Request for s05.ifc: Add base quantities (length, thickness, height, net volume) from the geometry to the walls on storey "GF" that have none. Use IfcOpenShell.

First a look at what the model holds.

```python
import ifcopenshell
import ifcopenshell.util.element
import ifcopenshell.util.unit

model = ifcopenshell.open("s05.ifc")
print(model.schema)
for unit_type in ("LENGTHUNIT", "AREAUNIT", "VOLUMEUNIT"):
    print(unit_type, ifcopenshell.util.unit.calculate_unit_scale(model, unit_type))
storey = next(s for s in model.by_type("IfcBuildingStorey") if s.Name == "GF")
walls = [e for e in ifcopenshell.util.element.get_decomposition(storey) if e.is_a("IfcWall")]
for e in sorted(walls, key=lambda e: e.id()):
    print(e.id(), e.is_a(), e.Name, list(ifcopenshell.util.element.get_psets(e, qtos_only=True)), sep=" | ")
```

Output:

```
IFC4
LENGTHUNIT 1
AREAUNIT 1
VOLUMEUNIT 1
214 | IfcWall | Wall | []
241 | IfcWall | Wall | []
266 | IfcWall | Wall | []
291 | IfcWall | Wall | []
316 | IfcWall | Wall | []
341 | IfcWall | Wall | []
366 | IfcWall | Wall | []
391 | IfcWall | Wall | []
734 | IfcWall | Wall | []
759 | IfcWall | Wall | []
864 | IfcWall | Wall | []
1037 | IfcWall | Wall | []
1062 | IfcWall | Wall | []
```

```python
import ifcopenshell
import ifcopenshell.api.pset
import ifcopenshell.geom
import ifcopenshell.util.element
import ifcopenshell.util.shape
import ifcopenshell.util.unit

model = ifcopenshell.open("s05.ifc")
unit_scale = ifcopenshell.util.unit.calculate_unit_scale(model)
volume_scale = ifcopenshell.util.unit.calculate_unit_scale(model, "VOLUMEUNIT")
settings = ifcopenshell.geom.settings()

storey = next(s for s in model.by_type("IfcBuildingStorey") if s.Name == "GF")
walls = [e for e in ifcopenshell.util.element.get_decomposition(storey) if e.is_a("IfcWall")]

for e in sorted(walls, key=lambda e: e.id()):
    if ifcopenshell.util.element.get_psets(e, qtos_only=True, should_inherit=False):
        continue
    # Geometry comes back in metres, in the element's own axes.
    shape = ifcopenshell.geom.create_shape(settings, e)
    values = {
        "Length": ifcopenshell.util.shape.get_x(shape.geometry) / unit_scale,
        "Width": ifcopenshell.util.shape.get_y(shape.geometry) / unit_scale,
        "Height": ifcopenshell.util.shape.get_z(shape.geometry) / unit_scale,
        "NetVolume": ifcopenshell.util.shape.get_volume(shape.geometry) / volume_scale,
    }
    qto = ifcopenshell.api.pset.add_qto(model, product=e, name="Qto_WallBaseQuantities")
    ifcopenshell.api.pset.edit_qto(model, qto=qto, properties=values)
    print(e.id(), {k: round(v, 3) for k, v in values.items()})

model.write("s05_rev.ifc")
```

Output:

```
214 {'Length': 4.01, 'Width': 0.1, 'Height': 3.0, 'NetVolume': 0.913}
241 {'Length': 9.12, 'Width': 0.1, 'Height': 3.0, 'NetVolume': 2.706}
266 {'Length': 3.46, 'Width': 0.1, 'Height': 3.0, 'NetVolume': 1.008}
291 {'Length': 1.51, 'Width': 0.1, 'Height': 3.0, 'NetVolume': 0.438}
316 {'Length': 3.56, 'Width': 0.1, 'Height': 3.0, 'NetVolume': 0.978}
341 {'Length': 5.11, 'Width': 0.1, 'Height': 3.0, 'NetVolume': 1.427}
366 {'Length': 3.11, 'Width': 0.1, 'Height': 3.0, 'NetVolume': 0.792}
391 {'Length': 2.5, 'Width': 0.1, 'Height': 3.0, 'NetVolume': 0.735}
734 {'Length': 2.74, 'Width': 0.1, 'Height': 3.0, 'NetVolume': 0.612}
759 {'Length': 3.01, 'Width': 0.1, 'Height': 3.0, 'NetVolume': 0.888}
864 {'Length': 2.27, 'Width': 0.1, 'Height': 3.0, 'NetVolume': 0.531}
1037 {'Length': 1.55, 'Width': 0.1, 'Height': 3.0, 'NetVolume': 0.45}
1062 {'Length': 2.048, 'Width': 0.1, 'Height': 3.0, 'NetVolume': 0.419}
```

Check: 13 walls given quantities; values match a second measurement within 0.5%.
